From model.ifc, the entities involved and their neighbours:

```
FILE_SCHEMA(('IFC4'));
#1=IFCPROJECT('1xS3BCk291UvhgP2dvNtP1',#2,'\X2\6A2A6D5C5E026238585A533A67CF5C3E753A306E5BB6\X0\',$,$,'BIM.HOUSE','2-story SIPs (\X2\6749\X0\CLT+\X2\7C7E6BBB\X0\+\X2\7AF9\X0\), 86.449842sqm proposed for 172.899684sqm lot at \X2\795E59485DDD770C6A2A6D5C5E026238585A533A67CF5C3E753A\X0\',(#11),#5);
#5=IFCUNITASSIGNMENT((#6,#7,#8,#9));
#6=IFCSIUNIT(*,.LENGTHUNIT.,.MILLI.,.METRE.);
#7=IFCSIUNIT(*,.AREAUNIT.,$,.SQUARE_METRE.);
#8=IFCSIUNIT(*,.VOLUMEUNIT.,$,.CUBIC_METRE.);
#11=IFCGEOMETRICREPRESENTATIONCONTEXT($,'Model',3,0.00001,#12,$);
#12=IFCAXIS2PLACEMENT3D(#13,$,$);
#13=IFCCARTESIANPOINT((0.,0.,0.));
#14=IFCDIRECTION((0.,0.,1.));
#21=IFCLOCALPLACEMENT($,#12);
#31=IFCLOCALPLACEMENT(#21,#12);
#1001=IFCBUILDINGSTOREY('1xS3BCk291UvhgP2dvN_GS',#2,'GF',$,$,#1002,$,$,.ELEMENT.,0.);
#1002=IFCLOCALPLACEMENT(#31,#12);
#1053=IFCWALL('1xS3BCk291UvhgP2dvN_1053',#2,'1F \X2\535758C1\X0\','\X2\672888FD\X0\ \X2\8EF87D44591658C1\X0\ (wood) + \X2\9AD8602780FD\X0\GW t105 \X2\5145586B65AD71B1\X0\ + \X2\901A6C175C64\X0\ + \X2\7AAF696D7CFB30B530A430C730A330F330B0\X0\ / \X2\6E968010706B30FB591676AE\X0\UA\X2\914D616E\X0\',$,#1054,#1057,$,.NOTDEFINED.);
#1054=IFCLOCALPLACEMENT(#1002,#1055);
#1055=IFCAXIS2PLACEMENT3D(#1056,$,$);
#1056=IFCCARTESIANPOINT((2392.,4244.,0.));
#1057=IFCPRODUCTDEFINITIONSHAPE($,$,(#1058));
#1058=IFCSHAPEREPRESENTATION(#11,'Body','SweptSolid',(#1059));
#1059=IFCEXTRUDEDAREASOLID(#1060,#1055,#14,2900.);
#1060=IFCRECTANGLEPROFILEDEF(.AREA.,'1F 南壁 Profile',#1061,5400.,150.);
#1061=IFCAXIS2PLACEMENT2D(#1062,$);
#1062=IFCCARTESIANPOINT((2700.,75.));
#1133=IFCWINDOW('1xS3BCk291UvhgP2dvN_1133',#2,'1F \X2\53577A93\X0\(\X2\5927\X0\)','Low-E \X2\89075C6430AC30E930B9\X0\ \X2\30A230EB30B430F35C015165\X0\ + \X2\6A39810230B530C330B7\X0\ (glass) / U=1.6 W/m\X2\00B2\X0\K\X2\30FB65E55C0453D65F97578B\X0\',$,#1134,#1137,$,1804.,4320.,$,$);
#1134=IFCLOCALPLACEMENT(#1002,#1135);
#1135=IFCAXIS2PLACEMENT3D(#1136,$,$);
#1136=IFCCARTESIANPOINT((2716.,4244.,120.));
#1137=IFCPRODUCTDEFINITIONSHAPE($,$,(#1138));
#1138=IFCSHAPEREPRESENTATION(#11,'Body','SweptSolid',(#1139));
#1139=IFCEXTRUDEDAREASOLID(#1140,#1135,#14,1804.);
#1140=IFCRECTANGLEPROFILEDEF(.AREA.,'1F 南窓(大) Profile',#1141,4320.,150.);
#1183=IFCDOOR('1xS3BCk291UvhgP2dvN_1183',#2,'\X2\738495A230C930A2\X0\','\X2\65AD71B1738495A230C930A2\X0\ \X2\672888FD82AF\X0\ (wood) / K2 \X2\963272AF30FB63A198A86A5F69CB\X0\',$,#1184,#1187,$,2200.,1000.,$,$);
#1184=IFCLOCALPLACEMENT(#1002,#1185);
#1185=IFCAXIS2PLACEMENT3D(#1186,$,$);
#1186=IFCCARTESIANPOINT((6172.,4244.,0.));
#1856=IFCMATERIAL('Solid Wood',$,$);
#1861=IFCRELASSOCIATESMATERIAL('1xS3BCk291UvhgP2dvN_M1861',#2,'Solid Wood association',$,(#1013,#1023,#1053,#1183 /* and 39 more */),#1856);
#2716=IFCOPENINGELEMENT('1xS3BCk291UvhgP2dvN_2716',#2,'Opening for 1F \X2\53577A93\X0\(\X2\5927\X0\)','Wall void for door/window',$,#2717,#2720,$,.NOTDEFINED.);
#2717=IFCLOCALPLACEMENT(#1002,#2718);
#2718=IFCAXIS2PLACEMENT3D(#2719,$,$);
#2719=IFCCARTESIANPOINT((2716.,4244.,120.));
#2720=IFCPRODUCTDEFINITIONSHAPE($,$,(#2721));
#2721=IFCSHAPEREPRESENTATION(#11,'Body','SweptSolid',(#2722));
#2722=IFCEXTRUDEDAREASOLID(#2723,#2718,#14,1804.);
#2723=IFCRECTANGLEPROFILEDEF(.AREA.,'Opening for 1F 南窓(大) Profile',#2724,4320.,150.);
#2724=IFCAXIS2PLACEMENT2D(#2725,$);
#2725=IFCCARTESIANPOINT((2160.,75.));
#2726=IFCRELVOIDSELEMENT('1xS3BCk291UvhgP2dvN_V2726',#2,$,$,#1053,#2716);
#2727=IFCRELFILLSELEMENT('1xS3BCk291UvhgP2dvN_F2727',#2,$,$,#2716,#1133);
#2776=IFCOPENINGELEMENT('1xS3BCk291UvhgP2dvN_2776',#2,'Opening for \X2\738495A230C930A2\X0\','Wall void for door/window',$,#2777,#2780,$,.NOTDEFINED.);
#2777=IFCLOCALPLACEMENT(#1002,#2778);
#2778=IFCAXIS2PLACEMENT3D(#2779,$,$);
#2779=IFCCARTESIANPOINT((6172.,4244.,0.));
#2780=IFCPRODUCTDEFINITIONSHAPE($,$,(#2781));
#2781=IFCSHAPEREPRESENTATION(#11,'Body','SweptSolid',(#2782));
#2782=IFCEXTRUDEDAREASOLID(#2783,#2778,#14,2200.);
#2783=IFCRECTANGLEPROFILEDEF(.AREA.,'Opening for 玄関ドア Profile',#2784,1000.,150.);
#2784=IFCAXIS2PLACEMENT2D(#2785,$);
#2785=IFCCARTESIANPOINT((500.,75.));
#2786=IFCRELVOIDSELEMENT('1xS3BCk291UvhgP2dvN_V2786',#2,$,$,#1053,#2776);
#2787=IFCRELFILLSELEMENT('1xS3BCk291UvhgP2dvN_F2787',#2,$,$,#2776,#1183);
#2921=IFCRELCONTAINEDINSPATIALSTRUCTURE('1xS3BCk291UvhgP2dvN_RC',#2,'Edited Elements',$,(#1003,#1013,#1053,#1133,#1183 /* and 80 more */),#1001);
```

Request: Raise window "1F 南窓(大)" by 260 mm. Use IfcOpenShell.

```python
import numpy as np
import ifcopenshell
import ifcopenshell.api.geometry
import ifcopenshell.util.placement
import ifcopenshell.util.unit

model = ifcopenshell.open("model.ifc")
unit_scale = ifcopenshell.util.unit.calculate_unit_scale(model)

window = model.by_id(1133)
opening = window.FillsVoids[0].RelatingOpeningElement
dz = 0.26 / unit_scale

shift = np.array([0.0, 0.0, dz])
# The window is not placed relative to its opening, so move both.
for product in (opening, window):
    matrix = ifcopenshell.util.placement.get_local_placement(product.ObjectPlacement)
    matrix[:3, 3] += shift
    ifcopenshell.api.geometry.edit_object_placement(model, product=product, matrix=matrix, is_si=False)

print(f"moved by {dz * unit_scale:+.3f} m")

model.write("model_v2.ifc")
```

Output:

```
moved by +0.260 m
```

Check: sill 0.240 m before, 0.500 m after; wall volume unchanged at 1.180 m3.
